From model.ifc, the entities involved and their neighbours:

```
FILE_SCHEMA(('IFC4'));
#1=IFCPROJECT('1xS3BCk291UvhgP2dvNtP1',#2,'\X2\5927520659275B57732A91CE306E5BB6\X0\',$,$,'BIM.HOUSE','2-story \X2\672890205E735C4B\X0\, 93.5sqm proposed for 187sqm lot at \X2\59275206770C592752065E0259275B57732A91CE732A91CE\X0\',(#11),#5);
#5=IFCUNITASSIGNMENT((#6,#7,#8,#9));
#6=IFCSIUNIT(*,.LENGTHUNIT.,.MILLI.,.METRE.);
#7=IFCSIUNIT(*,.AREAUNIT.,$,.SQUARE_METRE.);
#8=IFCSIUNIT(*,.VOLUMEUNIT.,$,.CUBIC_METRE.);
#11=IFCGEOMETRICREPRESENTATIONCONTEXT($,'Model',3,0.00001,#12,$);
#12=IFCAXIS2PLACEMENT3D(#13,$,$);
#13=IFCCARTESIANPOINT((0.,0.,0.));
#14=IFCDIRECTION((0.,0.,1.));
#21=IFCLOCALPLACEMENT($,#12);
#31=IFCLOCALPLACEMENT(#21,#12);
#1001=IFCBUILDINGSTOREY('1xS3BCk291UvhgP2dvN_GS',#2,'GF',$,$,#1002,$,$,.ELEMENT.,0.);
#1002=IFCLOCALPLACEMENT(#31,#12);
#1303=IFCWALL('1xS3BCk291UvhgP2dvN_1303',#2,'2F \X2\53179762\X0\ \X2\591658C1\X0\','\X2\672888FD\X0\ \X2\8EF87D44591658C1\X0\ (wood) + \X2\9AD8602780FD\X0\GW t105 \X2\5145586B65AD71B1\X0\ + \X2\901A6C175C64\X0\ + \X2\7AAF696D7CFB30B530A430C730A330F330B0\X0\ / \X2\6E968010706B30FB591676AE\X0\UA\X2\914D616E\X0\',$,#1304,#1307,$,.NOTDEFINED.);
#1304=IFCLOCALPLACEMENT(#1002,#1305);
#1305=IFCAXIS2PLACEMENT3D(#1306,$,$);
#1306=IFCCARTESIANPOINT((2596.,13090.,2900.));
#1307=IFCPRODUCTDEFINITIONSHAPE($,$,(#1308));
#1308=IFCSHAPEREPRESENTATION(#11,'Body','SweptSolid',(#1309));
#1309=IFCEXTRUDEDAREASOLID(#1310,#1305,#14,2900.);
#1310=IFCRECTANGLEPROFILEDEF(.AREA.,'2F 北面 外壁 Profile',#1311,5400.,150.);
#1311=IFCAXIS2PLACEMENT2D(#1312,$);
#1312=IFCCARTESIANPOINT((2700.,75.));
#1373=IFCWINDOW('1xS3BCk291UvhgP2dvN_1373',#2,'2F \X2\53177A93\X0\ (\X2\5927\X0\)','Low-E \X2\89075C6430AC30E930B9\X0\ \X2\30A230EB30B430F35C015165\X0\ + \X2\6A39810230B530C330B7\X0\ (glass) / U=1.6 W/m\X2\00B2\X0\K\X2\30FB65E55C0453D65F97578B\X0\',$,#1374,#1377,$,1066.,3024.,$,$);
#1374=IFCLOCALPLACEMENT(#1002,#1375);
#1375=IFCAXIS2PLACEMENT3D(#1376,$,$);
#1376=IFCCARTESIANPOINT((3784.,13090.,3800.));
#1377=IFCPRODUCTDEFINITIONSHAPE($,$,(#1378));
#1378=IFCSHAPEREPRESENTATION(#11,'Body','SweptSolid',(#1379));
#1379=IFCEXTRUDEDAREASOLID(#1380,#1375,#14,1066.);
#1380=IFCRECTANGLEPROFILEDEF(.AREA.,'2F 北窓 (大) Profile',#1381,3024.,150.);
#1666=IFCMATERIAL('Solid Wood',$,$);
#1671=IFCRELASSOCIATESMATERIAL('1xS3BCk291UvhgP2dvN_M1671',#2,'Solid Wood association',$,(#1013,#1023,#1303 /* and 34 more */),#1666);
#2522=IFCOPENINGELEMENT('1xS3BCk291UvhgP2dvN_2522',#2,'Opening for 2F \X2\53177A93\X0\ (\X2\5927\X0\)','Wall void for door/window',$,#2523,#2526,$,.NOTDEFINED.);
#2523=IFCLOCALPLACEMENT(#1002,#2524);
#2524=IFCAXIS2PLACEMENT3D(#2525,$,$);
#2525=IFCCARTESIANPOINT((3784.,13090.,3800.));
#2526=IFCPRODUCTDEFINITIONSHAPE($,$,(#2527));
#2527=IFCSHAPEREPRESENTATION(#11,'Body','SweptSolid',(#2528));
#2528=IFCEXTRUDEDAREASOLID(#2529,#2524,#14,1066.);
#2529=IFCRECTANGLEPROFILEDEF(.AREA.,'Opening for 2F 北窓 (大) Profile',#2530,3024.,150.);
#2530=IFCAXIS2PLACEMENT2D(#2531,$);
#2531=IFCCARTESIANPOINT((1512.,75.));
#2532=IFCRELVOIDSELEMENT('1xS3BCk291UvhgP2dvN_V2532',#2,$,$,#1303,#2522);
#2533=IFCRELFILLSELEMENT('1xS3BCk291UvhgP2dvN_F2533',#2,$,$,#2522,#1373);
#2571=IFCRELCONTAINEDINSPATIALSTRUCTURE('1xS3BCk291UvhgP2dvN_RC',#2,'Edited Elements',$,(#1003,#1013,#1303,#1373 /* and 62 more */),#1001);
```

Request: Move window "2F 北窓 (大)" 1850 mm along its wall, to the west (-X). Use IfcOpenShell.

```python
import ifcopenshell
import ifcopenshell.api.geometry
import ifcopenshell.util.placement

model = ifcopenshell.open("model.ifc")

window = model.by_guid("1xS3BCk291UvhgP2dvN_1373")
opening = window.FillsVoids[0].RelatingOpeningElement
wall = opening.VoidsElements[0].RelatingBuildingElement

wall_matrix = ifcopenshell.util.placement.get_local_placement(wall.ObjectPlacement)
shift = wall_matrix[:3, 0] * -1850.0
before = ifcopenshell.util.placement.get_local_placement(window.ObjectPlacement)[:3, 3].copy()

# The window is not placed relative to its opening, so move both.
for product in (opening, window):
    matrix = ifcopenshell.util.placement.get_local_placement(product.ObjectPlacement)
    matrix[:3, 3] += shift
    ifcopenshell.api.geometry.edit_object_placement(model, product=product, matrix=matrix, is_si=False)

after = ifcopenshell.util.placement.get_local_placement(window.ObjectPlacement)[:3, 3]
print("window moved by", (after - before).round(3) + 0.0)

model.write("model_v2.ifc")
```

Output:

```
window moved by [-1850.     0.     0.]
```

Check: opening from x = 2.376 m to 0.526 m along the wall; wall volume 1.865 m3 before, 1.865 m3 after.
